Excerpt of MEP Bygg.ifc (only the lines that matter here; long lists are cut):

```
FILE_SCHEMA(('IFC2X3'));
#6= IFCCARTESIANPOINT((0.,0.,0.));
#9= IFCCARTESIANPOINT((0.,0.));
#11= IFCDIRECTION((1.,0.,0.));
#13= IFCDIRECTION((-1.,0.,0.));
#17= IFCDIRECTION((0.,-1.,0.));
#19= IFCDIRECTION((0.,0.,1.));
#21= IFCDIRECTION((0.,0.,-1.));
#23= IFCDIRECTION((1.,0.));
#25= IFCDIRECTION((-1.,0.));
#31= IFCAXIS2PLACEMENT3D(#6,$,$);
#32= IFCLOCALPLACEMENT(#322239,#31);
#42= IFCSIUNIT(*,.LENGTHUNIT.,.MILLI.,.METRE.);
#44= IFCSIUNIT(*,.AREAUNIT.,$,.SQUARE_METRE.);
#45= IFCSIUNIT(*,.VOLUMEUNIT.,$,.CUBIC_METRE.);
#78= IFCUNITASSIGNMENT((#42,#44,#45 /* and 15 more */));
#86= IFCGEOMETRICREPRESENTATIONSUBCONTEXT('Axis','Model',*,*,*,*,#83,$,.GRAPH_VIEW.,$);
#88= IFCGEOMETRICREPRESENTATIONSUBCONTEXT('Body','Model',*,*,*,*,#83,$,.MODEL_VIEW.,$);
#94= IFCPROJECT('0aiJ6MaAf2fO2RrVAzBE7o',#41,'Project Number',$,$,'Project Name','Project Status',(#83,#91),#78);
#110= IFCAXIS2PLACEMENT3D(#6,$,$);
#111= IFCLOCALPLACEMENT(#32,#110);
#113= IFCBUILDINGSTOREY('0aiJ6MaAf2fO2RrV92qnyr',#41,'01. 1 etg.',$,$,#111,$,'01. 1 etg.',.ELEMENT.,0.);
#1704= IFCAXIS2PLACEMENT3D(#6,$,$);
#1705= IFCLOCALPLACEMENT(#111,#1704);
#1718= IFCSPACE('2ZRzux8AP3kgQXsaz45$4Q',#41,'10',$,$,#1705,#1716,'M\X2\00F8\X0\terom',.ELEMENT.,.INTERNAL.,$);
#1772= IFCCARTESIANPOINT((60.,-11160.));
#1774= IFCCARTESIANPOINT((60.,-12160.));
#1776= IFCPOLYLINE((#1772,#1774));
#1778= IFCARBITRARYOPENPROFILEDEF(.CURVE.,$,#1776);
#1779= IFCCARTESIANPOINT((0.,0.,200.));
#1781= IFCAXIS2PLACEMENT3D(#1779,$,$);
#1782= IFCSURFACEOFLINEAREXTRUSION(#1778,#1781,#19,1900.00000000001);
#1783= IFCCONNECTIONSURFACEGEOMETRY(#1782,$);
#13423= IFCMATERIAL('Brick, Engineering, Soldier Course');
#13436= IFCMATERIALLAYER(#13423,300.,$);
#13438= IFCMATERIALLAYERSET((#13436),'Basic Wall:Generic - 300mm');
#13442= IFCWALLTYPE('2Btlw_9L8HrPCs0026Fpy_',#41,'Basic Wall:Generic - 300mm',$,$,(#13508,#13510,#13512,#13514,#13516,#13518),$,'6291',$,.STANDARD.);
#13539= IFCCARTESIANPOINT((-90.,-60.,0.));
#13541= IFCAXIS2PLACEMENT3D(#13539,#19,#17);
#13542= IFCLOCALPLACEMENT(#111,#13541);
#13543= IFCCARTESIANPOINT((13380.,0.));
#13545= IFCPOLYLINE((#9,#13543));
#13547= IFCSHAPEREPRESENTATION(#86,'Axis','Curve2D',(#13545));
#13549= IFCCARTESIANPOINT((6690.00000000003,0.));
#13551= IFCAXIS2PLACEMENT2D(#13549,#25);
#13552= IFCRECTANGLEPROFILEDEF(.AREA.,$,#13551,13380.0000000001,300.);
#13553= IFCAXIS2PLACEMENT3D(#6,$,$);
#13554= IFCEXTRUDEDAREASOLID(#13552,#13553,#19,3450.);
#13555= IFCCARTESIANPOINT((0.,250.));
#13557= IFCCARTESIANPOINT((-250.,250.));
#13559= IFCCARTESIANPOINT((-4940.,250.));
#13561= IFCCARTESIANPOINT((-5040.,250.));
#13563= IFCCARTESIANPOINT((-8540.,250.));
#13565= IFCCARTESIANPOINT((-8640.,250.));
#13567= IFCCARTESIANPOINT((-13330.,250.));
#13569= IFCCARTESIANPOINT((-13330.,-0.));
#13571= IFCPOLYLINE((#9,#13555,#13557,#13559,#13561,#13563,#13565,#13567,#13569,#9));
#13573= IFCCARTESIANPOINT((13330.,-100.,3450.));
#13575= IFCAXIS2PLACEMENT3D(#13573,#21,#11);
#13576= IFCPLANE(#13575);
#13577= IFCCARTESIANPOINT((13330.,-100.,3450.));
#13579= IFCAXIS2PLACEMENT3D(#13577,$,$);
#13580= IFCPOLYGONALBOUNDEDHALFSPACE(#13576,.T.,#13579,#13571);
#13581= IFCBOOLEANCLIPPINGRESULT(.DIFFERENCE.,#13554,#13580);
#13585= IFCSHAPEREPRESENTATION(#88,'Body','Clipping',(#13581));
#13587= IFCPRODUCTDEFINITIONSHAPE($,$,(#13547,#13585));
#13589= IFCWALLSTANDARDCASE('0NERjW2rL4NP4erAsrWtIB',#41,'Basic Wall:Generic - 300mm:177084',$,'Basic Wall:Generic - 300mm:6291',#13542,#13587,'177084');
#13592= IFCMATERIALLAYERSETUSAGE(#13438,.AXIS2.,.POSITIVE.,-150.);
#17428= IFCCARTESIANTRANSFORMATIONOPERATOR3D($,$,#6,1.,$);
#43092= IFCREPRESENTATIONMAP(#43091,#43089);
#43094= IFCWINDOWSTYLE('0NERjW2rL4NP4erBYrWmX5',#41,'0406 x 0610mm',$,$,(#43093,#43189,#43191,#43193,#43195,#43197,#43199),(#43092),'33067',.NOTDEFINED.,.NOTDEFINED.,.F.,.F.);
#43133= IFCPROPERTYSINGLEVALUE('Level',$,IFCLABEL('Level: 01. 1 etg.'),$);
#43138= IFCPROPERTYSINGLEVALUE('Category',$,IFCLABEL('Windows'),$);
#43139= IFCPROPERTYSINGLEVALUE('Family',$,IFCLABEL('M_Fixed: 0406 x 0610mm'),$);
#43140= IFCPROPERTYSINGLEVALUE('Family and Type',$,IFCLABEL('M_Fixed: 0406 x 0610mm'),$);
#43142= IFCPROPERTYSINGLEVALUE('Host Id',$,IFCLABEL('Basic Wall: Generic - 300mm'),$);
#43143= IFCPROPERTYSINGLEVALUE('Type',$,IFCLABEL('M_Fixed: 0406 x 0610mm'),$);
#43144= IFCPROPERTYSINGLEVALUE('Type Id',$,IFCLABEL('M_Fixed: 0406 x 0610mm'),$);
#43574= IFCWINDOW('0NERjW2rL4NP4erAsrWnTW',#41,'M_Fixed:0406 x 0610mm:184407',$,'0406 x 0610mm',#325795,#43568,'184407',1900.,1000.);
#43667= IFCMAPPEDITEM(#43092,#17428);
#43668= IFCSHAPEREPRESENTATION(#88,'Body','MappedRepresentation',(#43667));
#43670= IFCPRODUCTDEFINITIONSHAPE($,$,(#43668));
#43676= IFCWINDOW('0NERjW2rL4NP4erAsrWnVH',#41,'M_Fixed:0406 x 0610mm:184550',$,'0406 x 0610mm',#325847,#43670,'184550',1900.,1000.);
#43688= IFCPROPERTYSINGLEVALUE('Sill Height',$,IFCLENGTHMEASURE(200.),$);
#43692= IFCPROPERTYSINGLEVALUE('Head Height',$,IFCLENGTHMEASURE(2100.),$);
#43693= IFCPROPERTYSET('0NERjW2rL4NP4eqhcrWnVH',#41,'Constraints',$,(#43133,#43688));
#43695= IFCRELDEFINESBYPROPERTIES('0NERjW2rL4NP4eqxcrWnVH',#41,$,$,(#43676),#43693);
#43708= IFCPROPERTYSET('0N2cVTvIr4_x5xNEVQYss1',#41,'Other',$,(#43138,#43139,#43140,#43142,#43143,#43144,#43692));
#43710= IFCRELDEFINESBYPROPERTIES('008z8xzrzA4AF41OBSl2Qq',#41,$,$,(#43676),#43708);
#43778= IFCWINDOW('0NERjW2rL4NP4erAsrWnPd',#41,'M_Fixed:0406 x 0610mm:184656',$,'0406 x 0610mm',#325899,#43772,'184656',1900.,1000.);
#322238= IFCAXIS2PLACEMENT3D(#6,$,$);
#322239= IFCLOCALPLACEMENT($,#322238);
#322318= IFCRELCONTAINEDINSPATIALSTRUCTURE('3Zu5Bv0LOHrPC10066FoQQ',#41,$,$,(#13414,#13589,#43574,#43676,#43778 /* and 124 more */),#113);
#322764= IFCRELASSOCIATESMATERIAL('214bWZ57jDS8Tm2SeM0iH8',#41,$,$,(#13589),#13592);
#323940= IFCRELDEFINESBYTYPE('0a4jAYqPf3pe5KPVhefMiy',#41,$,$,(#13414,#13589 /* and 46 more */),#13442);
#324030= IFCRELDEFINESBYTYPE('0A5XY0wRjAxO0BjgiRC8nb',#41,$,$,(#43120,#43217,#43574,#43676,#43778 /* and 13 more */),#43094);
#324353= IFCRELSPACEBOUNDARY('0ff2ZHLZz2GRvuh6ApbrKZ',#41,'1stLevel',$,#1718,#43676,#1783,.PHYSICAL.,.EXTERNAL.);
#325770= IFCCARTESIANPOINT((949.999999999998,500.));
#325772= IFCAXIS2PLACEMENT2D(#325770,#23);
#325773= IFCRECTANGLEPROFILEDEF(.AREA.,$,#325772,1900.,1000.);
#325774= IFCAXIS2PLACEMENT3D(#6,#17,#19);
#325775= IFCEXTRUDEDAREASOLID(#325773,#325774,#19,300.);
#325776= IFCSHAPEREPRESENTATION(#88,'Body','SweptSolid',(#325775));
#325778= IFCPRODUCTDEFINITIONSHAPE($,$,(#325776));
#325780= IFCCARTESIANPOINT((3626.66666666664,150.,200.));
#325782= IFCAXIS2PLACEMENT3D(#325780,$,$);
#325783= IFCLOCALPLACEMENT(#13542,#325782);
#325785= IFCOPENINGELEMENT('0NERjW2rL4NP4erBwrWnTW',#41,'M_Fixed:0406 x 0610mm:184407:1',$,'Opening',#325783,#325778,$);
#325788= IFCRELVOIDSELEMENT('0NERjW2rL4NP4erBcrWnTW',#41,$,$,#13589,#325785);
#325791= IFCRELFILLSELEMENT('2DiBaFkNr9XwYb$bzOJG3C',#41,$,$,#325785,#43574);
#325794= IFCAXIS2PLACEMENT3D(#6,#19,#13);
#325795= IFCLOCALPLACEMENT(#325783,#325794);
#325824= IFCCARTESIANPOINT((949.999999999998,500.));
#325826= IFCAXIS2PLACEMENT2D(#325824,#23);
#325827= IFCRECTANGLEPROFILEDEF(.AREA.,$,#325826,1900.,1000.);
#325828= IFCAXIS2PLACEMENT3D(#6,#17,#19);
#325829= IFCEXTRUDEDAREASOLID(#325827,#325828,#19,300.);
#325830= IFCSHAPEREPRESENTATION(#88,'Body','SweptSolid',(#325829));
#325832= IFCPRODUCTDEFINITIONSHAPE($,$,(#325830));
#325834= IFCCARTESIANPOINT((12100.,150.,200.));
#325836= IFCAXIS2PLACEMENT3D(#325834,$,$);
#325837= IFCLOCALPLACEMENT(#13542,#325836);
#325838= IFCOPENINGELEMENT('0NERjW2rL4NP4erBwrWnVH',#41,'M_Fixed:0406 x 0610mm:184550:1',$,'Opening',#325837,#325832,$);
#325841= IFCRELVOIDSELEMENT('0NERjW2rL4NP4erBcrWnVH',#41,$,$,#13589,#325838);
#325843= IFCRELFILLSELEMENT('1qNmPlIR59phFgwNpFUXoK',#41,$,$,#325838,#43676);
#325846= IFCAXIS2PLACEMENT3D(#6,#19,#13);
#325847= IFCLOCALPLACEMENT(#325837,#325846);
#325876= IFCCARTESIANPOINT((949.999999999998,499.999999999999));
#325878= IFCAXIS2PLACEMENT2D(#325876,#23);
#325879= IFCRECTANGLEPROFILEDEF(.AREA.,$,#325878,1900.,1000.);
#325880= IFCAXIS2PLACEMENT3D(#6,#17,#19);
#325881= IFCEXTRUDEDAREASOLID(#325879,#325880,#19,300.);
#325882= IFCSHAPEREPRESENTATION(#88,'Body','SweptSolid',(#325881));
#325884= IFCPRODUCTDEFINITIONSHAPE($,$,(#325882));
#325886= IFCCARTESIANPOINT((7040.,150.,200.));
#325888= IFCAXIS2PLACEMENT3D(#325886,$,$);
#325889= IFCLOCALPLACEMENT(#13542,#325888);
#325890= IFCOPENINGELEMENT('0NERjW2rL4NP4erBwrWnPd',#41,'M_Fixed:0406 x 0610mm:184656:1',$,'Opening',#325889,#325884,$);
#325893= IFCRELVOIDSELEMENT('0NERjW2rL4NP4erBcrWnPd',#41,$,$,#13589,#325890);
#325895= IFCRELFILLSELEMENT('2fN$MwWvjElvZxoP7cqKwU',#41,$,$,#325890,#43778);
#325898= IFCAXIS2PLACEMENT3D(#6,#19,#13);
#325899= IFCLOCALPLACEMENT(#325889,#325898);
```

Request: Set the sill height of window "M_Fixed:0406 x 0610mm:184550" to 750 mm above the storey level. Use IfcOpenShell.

```python
import numpy as np
import ifcopenshell
import ifcopenshell.api.geometry
import ifcopenshell.api.pset
import ifcopenshell.geom
import ifcopenshell.util.element
import ifcopenshell.util.placement
import ifcopenshell.util.shape
import ifcopenshell.util.unit

model = ifcopenshell.open("MEP Bygg.ifc")
unit_scale = ifcopenshell.util.unit.calculate_unit_scale(model)

window = model.by_guid("0NERjW2rL4NP4erAsrWnVH")
opening = window.FillsVoids[0].RelatingOpeningElement
storey = ifcopenshell.util.element.get_container(window, ifc_class="IfcBuildingStorey")
level = ifcopenshell.util.placement.get_local_placement(storey.ObjectPlacement)[2, 3]

# The opening's origin need not be at the sill, so measure its lowest point.
shape = ifcopenshell.geom.create_shape(ifcopenshell.geom.settings(), opening)
bottom = ifcopenshell.util.shape.get_shape_bottom_elevation(shape, shape.geometry) / unit_scale
dz = level + 750.0 - bottom

shift = np.array([0.0, 0.0, dz])
# The window is placed relative to its opening, so it follows when the opening moves.
matrix = ifcopenshell.util.placement.get_local_placement(opening.ObjectPlacement)
matrix[:3, 3] += shift
ifcopenshell.api.geometry.edit_object_placement(
    model, product=opening, matrix=matrix, is_si=False, should_transform_children=True
)

# Space boundary surfaces are stored in each space's coordinates; move them too.
for rel in window.ProvidesBoundaries:
    if not rel.ConnectionGeometry:
        continue
    surface = rel.ConnectionGeometry.SurfaceOnRelatingElement
    space_matrix = ifcopenshell.util.placement.get_local_placement(rel.RelatingSpace.ObjectPlacement)
    point = np.array(surface.Position.Location.Coordinates) + space_matrix[:3, :3].T @ shift
    surface.Position = model.createIfcAxis2Placement3D(
        model.createIfcCartesianPoint(point.tolist()), surface.Position.Axis, surface.Position.RefDirection
    )

# Keep the stored heights in step.
pset = model.by_id(ifcopenshell.util.element.get_pset(window, "Constraints", should_inherit=False)["id"])
ifcopenshell.api.pset.edit_pset(model, pset=pset, properties={
    "Sill Height": model.create_entity("IfcLengthMeasure", ifcopenshell.util.element.get_pset(window, "Constraints", "Sill Height") + dz),
})
pset = model.by_id(ifcopenshell.util.element.get_pset(window, "Other", should_inherit=False)["id"])
ifcopenshell.api.pset.edit_pset(model, pset=pset, properties={
    "Head Height": model.create_entity("IfcLengthMeasure", ifcopenshell.util.element.get_pset(window, "Other", "Head Height") + dz),
})

print(f"moved by {dz * unit_scale:+.3f} m")

model.write("MEP Bygg_updated.ifc")
```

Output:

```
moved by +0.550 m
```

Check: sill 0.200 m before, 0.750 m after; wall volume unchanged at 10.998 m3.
